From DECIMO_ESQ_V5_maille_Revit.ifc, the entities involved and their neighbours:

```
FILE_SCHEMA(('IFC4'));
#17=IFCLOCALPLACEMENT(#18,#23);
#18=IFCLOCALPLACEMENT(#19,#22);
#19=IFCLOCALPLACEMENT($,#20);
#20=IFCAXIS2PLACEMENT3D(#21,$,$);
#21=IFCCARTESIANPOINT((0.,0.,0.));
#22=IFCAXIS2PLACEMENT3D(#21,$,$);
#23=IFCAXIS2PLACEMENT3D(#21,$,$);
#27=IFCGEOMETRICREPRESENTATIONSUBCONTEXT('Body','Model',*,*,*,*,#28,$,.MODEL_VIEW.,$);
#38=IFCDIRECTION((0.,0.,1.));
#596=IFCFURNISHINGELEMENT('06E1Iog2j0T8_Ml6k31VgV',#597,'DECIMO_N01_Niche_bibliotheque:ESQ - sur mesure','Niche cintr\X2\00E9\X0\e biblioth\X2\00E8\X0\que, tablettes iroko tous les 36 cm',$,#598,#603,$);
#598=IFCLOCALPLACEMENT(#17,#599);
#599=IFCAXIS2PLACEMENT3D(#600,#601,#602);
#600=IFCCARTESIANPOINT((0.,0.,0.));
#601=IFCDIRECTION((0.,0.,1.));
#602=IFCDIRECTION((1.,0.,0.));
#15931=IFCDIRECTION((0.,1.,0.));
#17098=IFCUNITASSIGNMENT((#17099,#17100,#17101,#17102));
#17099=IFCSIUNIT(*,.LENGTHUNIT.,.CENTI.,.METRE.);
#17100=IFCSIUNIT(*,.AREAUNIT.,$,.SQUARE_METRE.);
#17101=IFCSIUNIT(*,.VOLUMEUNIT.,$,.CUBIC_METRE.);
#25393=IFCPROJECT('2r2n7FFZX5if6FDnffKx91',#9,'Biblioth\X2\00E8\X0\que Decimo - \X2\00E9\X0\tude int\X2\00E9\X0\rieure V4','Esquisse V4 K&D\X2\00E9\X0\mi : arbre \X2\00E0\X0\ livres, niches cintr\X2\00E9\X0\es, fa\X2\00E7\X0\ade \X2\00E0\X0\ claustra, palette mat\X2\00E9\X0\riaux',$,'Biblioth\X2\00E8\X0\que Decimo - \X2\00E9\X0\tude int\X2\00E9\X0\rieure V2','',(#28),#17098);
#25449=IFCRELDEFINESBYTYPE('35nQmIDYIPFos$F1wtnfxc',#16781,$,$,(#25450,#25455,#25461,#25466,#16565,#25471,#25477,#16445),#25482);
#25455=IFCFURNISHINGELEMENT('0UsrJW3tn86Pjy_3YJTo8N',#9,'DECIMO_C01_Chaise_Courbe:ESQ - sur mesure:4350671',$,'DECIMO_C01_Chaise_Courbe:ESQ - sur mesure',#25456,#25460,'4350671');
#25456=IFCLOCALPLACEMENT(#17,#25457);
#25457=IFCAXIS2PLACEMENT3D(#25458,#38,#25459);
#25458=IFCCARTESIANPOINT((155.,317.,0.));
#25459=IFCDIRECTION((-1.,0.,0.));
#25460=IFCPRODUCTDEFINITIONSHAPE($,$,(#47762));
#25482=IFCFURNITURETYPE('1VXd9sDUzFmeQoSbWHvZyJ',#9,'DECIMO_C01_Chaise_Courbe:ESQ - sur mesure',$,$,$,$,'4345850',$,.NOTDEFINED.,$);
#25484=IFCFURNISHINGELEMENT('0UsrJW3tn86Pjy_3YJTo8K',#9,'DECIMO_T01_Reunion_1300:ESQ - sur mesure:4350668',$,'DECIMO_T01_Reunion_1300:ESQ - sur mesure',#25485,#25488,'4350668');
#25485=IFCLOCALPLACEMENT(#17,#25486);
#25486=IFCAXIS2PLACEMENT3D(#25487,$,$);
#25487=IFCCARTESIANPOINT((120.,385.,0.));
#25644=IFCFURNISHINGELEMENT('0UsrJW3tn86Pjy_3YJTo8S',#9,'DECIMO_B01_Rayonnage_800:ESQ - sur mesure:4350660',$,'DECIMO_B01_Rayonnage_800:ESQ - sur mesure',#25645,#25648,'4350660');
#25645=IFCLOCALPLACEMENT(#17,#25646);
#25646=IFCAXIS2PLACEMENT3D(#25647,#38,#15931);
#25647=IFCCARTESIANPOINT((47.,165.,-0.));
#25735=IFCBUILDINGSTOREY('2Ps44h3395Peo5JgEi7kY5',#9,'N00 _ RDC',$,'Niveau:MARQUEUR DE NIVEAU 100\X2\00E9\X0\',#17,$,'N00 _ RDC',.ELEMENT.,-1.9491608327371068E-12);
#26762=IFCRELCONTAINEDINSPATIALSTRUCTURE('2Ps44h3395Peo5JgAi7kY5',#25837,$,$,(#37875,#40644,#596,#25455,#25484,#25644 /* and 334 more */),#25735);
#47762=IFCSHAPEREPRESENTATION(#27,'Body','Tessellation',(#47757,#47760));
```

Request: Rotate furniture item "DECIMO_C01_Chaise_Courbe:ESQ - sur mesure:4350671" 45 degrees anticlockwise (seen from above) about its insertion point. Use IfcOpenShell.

```python
import ifcopenshell
import ifcopenshell.api.geometry
import ifcopenshell.util.placement

model = ifcopenshell.open("DECIMO_ESQ_V5_maille_Revit.ifc")

item = model.by_id(25455)
matrix = ifcopenshell.util.placement.get_local_placement(item.ObjectPlacement)
matrix = matrix @ ifcopenshell.util.placement.rotation(45, "Z")
ifcopenshell.api.geometry.edit_object_placement(model, product=item, matrix=matrix, is_si=False)

print(ifcopenshell.util.placement.get_local_placement(item.ObjectPlacement).round(3) + 0.0)

model.write("DECIMO_ESQ_V5_maille_Revit_v2.ifc")
```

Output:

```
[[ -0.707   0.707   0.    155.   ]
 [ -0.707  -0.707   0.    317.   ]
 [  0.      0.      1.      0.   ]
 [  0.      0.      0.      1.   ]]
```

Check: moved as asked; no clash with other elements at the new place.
